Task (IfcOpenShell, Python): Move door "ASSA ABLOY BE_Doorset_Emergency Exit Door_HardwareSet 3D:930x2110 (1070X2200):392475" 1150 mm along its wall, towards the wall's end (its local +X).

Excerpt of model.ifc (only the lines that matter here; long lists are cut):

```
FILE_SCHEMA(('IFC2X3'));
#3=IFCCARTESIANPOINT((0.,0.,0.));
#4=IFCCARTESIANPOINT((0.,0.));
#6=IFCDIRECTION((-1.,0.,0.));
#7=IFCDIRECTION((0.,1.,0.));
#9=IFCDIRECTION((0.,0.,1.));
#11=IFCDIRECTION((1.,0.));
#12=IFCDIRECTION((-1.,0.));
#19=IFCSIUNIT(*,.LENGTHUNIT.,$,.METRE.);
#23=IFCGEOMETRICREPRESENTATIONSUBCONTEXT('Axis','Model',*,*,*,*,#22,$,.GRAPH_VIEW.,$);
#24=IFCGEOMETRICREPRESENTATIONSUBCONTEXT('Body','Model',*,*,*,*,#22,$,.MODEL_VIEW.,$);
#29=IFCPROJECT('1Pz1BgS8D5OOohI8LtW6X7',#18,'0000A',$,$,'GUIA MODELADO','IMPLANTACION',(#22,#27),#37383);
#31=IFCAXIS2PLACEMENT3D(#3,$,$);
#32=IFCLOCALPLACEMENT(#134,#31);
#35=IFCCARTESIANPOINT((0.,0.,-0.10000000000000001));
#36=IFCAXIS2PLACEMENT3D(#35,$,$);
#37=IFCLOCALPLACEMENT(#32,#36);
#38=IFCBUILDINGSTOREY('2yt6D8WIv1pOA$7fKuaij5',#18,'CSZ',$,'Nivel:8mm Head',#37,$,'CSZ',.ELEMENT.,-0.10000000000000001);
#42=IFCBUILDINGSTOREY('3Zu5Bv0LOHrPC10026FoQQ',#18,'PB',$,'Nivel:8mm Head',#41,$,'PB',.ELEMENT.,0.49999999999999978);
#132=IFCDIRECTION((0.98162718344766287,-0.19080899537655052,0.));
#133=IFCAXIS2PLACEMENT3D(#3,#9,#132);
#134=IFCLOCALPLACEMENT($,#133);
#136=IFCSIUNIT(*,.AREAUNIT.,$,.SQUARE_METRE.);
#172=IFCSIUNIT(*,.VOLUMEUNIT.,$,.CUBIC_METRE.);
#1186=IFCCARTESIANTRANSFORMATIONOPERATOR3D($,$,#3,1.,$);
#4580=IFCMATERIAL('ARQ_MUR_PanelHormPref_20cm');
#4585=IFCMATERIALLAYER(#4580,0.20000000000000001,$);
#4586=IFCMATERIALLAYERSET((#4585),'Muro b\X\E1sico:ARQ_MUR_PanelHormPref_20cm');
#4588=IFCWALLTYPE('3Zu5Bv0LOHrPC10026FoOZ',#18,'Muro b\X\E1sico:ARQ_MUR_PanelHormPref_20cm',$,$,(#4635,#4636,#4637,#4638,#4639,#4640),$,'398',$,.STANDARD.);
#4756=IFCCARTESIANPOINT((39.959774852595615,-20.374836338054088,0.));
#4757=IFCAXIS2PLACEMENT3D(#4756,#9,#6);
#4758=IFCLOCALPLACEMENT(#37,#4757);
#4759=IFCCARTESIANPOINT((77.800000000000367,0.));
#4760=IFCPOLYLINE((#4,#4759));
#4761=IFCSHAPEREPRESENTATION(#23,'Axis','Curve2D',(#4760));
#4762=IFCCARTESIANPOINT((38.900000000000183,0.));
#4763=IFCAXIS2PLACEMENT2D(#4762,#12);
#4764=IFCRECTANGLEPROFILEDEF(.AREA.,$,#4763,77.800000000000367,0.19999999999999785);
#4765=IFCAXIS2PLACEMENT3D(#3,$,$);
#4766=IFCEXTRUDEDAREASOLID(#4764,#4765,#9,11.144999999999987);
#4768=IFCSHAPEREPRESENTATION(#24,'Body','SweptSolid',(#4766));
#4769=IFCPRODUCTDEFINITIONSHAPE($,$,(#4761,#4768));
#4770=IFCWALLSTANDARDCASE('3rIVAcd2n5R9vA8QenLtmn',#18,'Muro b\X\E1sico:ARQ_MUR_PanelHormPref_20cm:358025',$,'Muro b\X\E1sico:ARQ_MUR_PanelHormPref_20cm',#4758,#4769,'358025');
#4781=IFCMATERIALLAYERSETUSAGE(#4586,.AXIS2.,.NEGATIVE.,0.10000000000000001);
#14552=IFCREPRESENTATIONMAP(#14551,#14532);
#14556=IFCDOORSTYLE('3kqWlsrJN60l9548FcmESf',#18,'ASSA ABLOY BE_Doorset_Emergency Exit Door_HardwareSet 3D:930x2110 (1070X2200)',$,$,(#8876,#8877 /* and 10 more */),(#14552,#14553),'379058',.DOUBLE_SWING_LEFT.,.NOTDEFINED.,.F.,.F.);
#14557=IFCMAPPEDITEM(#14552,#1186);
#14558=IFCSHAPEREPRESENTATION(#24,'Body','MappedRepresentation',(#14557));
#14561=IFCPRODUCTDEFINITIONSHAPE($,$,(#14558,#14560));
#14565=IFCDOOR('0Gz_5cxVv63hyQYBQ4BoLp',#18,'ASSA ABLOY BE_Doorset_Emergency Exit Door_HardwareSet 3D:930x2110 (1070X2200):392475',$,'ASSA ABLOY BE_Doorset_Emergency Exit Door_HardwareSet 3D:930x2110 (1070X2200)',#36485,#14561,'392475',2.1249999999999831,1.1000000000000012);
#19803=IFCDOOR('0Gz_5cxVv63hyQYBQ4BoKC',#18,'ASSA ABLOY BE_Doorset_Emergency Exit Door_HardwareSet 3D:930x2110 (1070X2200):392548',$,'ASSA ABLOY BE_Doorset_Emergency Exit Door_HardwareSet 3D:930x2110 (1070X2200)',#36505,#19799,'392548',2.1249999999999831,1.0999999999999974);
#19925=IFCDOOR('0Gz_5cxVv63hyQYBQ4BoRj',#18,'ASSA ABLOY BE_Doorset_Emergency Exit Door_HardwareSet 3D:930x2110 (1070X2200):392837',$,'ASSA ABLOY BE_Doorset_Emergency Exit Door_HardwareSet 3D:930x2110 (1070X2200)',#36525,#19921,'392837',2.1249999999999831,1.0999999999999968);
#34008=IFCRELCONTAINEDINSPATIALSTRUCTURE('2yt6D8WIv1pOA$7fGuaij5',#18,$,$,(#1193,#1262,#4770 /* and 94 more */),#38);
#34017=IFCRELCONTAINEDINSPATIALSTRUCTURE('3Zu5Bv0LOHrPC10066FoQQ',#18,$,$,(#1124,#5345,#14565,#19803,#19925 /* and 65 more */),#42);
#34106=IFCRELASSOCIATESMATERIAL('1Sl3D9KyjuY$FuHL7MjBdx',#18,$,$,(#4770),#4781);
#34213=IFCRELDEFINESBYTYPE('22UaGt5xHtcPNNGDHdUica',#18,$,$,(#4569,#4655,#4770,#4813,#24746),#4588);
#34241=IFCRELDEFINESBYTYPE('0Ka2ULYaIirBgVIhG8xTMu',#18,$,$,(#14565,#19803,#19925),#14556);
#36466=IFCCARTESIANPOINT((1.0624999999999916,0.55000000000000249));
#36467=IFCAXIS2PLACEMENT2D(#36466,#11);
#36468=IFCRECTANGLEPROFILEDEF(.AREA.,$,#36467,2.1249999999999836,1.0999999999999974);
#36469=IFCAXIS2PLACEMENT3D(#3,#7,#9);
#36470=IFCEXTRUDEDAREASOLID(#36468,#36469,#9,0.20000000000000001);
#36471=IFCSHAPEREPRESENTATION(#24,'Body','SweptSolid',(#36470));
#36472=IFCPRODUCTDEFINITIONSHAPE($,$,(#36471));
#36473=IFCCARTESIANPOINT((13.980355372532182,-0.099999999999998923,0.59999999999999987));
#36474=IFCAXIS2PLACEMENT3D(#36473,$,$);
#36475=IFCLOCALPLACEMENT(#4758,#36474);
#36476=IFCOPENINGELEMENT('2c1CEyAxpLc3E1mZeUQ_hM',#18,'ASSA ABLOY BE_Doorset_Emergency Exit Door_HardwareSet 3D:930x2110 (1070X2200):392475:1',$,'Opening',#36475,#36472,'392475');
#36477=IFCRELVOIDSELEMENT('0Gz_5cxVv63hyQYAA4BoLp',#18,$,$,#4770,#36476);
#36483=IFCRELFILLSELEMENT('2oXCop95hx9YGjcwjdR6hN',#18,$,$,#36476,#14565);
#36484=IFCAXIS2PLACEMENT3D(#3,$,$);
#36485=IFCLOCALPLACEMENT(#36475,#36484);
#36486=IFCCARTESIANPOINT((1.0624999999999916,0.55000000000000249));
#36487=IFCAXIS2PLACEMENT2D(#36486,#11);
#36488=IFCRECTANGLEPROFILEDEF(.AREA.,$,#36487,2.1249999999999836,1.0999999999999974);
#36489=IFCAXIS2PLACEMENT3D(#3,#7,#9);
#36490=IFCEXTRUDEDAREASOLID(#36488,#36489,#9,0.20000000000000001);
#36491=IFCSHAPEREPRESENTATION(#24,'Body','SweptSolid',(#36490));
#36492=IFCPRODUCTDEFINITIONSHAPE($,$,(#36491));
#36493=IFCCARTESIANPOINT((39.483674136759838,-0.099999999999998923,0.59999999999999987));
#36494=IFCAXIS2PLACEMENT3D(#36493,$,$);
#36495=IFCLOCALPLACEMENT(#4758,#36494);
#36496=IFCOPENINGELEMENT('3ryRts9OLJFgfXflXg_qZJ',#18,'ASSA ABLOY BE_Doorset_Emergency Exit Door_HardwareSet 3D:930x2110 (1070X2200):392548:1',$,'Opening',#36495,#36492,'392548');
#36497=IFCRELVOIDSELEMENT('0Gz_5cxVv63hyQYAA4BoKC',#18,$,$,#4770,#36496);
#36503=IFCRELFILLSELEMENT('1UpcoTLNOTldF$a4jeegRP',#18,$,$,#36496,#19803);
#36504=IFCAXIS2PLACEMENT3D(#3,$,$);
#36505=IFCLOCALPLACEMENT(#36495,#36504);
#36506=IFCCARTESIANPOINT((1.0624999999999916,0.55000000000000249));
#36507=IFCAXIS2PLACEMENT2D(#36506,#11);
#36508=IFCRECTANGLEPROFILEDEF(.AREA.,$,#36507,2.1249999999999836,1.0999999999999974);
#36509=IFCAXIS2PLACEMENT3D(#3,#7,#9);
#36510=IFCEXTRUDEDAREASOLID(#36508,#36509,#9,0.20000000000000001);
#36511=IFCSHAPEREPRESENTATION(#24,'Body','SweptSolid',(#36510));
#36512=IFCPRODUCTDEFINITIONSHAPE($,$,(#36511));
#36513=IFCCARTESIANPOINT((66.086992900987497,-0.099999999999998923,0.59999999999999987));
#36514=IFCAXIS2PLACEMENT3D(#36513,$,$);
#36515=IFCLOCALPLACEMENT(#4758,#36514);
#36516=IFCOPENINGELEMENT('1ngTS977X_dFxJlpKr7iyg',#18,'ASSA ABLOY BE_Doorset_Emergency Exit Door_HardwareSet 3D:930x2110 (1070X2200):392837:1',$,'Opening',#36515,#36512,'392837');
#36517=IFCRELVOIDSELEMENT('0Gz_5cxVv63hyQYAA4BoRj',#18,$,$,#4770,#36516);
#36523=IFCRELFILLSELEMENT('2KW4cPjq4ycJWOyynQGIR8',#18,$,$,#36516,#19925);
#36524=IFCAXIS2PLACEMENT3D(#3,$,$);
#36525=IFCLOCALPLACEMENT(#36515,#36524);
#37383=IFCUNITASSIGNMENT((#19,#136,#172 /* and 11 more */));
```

```python
import ifcopenshell
import ifcopenshell.api.geometry
import ifcopenshell.util.placement

model = ifcopenshell.open("model.ifc")

door = model.by_guid("0Gz_5cxVv63hyQYBQ4BoLp")
opening = door.FillsVoids[0].RelatingOpeningElement
wall = opening.VoidsElements[0].RelatingBuildingElement

wall_matrix = ifcopenshell.util.placement.get_local_placement(wall.ObjectPlacement)
shift = wall_matrix[:3, 0] * 1.15
before = ifcopenshell.util.placement.get_local_placement(door.ObjectPlacement)[:3, 3].copy()

# The door is placed relative to its opening, so it follows when the opening moves.
matrix = ifcopenshell.util.placement.get_local_placement(opening.ObjectPlacement)
matrix[:3, 3] += shift
ifcopenshell.api.geometry.edit_object_placement(
    model, product=opening, matrix=matrix, is_si=False, should_transform_children=True
)

after = ifcopenshell.util.placement.get_local_placement(door.ObjectPlacement)[:3, 3]
print("door moved by", (after - before).round(3) + 0.0)

model.write("model_updated.ifc")
```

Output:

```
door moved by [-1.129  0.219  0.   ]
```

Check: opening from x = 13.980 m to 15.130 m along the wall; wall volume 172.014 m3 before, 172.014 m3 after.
